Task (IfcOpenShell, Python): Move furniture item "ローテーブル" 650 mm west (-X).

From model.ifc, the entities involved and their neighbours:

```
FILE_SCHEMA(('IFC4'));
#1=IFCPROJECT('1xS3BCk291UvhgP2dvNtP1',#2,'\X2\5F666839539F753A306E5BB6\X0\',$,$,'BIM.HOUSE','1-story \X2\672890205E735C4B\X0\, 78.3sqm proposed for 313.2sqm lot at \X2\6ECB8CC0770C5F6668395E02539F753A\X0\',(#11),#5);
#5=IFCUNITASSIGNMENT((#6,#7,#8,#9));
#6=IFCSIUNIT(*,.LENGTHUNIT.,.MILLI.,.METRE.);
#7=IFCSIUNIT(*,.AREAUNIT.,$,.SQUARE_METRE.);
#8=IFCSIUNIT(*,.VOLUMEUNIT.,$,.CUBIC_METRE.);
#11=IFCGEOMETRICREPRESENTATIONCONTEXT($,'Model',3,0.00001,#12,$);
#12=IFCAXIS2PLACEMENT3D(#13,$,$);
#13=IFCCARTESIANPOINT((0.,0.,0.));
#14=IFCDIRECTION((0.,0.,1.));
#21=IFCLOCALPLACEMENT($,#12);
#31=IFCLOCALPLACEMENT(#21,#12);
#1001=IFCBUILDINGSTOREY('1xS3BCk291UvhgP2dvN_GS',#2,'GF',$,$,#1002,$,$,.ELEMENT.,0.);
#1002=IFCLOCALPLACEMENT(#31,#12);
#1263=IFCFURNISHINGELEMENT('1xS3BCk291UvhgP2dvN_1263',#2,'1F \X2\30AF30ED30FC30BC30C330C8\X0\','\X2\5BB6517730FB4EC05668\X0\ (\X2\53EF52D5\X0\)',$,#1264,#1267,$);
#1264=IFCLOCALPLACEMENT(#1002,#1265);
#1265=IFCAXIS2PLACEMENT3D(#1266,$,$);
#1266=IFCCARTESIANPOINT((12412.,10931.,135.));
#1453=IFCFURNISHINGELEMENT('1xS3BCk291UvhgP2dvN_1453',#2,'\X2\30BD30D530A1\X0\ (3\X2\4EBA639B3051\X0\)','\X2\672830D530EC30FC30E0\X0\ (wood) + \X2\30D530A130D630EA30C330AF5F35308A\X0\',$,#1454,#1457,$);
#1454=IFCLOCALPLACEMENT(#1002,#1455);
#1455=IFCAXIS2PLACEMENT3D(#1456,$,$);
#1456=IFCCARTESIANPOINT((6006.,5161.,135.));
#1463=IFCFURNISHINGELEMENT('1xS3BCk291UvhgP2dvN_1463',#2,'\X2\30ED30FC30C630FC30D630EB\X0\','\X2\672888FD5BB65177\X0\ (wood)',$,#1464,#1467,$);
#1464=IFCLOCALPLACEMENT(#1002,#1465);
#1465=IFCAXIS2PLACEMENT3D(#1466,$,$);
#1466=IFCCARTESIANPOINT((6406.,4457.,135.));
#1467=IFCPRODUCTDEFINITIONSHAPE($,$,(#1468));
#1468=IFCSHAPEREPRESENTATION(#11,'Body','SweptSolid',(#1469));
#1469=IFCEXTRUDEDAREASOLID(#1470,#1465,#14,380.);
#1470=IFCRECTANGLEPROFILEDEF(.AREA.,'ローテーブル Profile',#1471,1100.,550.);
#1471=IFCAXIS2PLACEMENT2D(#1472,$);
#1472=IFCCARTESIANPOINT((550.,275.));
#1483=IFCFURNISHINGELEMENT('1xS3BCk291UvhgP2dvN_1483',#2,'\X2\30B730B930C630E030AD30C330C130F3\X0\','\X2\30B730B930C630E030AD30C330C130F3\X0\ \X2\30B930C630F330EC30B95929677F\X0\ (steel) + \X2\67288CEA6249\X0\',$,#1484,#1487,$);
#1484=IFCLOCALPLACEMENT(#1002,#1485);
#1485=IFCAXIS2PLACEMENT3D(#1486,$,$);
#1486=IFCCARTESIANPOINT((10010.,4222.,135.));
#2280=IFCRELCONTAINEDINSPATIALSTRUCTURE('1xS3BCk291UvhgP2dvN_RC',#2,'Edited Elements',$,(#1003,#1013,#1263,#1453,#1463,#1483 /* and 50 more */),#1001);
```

```python
import ifcopenshell
import ifcopenshell.api.geometry
import ifcopenshell.util.placement
import ifcopenshell.util.unit

model = ifcopenshell.open("model.ifc")
unit_scale = ifcopenshell.util.unit.calculate_unit_scale(model)

item = model.by_guid("1xS3BCk291UvhgP2dvN_1463")
matrix = ifcopenshell.util.placement.get_local_placement(item.ObjectPlacement)
matrix[0, 3] -= 0.65 / unit_scale
ifcopenshell.api.geometry.edit_object_placement(model, product=item, matrix=matrix, is_si=False)

print(ifcopenshell.util.placement.get_local_placement(item.ObjectPlacement).round(3) + 0.0)

model.write("model_updated.ifc")
```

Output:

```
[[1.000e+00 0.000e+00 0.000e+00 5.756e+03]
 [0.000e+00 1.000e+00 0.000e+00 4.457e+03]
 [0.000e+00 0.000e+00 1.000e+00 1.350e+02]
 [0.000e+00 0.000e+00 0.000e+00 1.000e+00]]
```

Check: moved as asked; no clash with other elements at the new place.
